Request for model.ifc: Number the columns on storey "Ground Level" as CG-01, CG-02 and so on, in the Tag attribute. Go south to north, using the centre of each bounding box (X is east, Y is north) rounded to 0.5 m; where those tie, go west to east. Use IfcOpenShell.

First a look at what the model holds.

```python
import ifcopenshell
import ifcopenshell.util.element
import ifcopenshell.util.placement

model = ifcopenshell.open("model.ifc")
print(model.schema)
storey = next(s for s in model.by_type("IfcBuildingStorey") if s.Name == "Ground Level")
columns = [e for e in ifcopenshell.util.element.get_decomposition(storey) if e.is_a("IfcColumn")]
for e in sorted(columns, key=lambda e: e.id()):
    origin = ifcopenshell.util.placement.get_local_placement(e.ObjectPlacement)[:3, 3]
    print(e.id(), e.Tag, e.Name, origin.round(2) + 0.0, sep=" | ")
```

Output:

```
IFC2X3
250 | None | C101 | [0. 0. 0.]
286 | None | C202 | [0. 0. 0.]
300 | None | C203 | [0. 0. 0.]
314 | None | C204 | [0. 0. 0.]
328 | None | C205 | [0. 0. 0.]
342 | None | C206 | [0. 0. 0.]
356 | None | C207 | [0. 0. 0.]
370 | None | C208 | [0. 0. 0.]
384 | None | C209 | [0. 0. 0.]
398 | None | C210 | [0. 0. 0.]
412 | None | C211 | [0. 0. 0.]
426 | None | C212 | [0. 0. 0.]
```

```python
import ifcopenshell
import ifcopenshell.geom
import ifcopenshell.util.element
import ifcopenshell.util.shape

model = ifcopenshell.open("model.ifc")
settings = ifcopenshell.geom.settings()
settings.set("use-world-coords", True)


def centre(element):
    shape = ifcopenshell.geom.create_shape(settings, element)
    return ifcopenshell.util.shape.get_bbox_centroid(shape.geometry)


storey = next(s for s in model.by_type("IfcBuildingStorey") if s.Name == "Ground Level")
columns = [e for e in ifcopenshell.util.element.get_decomposition(storey) if e.is_a("IfcColumn")]

# Insertion points can sit at a corner or the storey origin, so sort by the geometry (in metres).
centres = {e: centre(e) for e in columns}
columns.sort(key=lambda e: (round(centres[e][1] / 0.5), centres[e][0]))

for i, e in enumerate(columns, start=1):
    number = f"CG-{i:02d}"
    e.Tag = number
    print(e.id(), number)

model.write("model_rev.ifc")
```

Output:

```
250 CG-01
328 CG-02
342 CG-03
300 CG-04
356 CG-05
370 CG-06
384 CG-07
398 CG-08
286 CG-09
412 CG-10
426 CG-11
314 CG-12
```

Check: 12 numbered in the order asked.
